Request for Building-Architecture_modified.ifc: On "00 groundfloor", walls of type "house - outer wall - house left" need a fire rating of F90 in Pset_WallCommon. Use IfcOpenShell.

First a look at what the model holds.

```python
import ifcopenshell
import ifcopenshell.util.element

model = ifcopenshell.open("Building-Architecture_modified.ifc")
print(model.schema)
storey = next(s for s in model.by_type("IfcBuildingStorey") if s.Name == "00 groundfloor")
walls = [e for e in ifcopenshell.util.element.get_decomposition(storey) if e.is_a("IfcWall")]
seen = {}
for e in walls:
    element_type = ifcopenshell.util.element.get_type(e)
    key = (element_type.Name if element_type != e and element_type else None, ifcopenshell.util.element.get_pset(e, "Pset_WallCommon", "FireRating"))
    seen[key] = seen.get(key, 0) + 1
for (name, value), count in sorted(seen.items(), key=str):
    print(count, "x", name, "|", value)
```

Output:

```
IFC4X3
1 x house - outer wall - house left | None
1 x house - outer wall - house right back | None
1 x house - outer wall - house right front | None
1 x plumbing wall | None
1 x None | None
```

```python
import ifcopenshell
import ifcopenshell.api.pset
import ifcopenshell.util.element

model = ifcopenshell.open("Building-Architecture_modified.ifc")

storey = next(s for s in model.by_type("IfcBuildingStorey") if s.Name == "00 groundfloor")
walls = [e for e in ifcopenshell.util.element.get_decomposition(storey) if e.is_a("IfcWall")]

count = 0
for e in walls:
    element_type = ifcopenshell.util.element.get_type(e)
    if element_type in (None, e) or element_type.Name != "house - outer wall - house left":
        continue
    # add_pset returns the element's existing set when there is one.
    pset = ifcopenshell.api.pset.add_pset(model, product=e, name="Pset_WallCommon")
    ifcopenshell.api.pset.edit_pset(model, pset=pset, properties={"FireRating": "F90"})
    count += 1

print(count, "walls updated")

model.write("Building-Architecture_modified-out.ifc")
```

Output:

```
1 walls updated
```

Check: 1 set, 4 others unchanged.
